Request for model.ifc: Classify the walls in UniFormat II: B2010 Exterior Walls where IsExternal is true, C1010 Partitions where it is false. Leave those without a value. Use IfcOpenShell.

First a look at what the model holds.

```python
import ifcopenshell
import ifcopenshell.util.element

model = ifcopenshell.open("model.ifc")
print(model.schema)
print("classifications:", [c.Name for c in model.by_type("IfcClassification")])
values = [ifcopenshell.util.element.get_pset(e, "Pset_WallCommon", "IsExternal") for e in model.by_type("IfcWall")]
for value in (True, False, None):
    print("IsExternal", value, values.count(value))
```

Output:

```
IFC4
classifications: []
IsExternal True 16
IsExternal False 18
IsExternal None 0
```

```python
import ifcopenshell
import ifcopenshell.api.classification
import ifcopenshell.util.element

model = ifcopenshell.open("model.ifc")

system = ifcopenshell.api.classification.add_classification(model, classification="UniFormat II")

walls = model.by_type("IfcWall")
external = {e: ifcopenshell.util.element.get_pset(e, "Pset_WallCommon", "IsExternal") for e in walls}
for flag, code, name in ((True, "B2010", "Exterior Walls"), (False, "C1010", "Partitions")):
    products = [e for e in walls if external[e] is flag]
    ifcopenshell.api.classification.add_reference(
        model, products=products, classification=system, identification=code, name=name
    )
    print(code, len(products))

model.write("model-out.ifc")
```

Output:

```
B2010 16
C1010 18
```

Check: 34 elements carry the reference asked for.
